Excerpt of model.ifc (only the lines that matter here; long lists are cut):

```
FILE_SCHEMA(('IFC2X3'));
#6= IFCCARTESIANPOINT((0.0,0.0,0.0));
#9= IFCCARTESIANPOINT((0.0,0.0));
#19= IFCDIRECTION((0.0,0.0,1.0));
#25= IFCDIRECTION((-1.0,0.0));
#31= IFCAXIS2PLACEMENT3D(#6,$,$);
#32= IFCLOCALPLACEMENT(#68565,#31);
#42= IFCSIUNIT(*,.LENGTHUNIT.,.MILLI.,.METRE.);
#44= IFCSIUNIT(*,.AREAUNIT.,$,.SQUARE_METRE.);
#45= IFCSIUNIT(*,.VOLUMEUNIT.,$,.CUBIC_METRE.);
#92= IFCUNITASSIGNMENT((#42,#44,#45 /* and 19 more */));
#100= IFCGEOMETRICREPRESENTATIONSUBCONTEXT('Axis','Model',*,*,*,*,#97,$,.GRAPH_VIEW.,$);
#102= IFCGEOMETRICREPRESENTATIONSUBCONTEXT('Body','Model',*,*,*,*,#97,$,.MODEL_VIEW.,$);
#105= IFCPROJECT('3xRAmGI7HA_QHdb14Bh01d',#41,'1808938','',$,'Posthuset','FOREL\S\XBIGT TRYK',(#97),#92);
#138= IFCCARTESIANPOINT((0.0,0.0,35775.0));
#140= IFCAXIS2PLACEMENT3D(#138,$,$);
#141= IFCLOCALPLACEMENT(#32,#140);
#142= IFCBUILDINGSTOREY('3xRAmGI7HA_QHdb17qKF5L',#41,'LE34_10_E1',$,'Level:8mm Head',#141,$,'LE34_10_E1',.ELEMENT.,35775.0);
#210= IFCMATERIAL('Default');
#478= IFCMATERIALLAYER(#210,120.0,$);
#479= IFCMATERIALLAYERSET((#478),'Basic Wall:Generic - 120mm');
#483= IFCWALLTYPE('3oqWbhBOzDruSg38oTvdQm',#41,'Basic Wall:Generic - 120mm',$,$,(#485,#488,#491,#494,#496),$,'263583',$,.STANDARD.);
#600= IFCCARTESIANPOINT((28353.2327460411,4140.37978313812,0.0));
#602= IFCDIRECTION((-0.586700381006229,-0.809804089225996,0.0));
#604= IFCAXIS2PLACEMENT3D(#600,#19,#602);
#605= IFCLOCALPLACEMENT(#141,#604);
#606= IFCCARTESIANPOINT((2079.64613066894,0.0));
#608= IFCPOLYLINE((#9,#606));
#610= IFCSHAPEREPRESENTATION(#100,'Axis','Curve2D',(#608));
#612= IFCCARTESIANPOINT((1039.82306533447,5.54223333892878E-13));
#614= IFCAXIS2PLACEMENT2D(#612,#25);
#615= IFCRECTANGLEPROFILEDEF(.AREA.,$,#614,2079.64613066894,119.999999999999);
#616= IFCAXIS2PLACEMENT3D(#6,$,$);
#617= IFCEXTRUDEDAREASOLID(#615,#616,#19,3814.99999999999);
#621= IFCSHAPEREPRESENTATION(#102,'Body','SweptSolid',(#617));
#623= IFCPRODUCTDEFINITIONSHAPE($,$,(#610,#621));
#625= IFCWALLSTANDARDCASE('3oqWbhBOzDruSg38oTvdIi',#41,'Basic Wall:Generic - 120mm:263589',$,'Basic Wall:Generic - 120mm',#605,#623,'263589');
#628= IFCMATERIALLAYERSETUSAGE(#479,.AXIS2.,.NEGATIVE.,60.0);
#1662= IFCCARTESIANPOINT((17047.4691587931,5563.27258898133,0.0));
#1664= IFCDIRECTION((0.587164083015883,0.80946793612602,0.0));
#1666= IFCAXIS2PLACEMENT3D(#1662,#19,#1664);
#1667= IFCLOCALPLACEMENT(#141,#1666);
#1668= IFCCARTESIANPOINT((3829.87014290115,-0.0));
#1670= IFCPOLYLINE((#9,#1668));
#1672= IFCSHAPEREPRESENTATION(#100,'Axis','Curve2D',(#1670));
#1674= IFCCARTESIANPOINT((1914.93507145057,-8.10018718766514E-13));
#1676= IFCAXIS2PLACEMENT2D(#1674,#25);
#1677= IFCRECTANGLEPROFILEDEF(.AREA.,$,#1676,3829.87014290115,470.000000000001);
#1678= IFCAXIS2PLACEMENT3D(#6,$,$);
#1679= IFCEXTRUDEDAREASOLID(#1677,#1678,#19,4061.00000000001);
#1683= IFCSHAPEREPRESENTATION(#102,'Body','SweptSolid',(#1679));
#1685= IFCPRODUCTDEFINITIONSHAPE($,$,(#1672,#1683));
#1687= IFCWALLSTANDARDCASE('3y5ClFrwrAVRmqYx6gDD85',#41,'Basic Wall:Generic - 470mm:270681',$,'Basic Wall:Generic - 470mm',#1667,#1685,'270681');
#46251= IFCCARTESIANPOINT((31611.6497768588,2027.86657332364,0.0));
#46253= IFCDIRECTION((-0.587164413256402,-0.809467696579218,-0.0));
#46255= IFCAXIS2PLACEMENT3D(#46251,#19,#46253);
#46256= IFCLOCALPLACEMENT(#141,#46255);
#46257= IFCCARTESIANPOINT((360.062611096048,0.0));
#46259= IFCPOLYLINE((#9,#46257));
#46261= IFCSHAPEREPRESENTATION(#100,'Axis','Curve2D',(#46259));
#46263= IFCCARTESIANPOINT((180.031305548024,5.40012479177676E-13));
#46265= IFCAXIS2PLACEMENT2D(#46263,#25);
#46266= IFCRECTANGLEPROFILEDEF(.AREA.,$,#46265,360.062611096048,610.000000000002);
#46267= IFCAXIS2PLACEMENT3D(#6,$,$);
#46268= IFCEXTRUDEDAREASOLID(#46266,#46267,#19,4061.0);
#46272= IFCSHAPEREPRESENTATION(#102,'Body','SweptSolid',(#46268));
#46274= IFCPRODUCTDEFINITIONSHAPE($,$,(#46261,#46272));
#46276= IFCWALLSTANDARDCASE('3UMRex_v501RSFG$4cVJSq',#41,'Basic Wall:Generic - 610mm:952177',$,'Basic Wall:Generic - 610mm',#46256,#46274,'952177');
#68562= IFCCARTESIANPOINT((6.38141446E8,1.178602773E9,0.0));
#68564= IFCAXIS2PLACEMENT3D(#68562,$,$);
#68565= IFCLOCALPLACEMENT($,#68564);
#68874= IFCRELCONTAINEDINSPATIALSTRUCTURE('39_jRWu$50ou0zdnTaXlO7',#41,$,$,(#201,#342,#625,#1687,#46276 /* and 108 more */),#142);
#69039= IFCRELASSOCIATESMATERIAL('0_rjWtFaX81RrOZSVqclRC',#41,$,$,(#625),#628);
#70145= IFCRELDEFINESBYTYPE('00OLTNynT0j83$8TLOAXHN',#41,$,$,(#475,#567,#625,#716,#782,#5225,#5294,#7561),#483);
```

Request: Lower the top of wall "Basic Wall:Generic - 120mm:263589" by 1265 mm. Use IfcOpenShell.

```python
import ifcopenshell
import ifcopenshell.geom
import ifcopenshell.util.representation
import ifcopenshell.util.shape
import ifcopenshell.util.unit

model = ifcopenshell.open("model.ifc")
unit_scale = ifcopenshell.util.unit.calculate_unit_scale(model)
settings = ifcopenshell.geom.settings()


def volume(element):
    """Net volume in cubic metres, openings subtracted."""
    shape = ifcopenshell.geom.create_shape(settings, element)
    return ifcopenshell.util.shape.get_volume(shape.geometry)


wall = model.by_id(625)
before = volume(wall)

body = ifcopenshell.util.representation.get_representation(wall, "Model", "Body")
solid = body.Items[0]
old_height = solid.Depth
solid.Depth -= 1.265 / unit_scale
after = volume(wall)

print(f"height {old_height:g} -> {solid.Depth:g}, volume {before:.3f} -> {after:.3f} m3")

model.write("model_rev.ifc")
```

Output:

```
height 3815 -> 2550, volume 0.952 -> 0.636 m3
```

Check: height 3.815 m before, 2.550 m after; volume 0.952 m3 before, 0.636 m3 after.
